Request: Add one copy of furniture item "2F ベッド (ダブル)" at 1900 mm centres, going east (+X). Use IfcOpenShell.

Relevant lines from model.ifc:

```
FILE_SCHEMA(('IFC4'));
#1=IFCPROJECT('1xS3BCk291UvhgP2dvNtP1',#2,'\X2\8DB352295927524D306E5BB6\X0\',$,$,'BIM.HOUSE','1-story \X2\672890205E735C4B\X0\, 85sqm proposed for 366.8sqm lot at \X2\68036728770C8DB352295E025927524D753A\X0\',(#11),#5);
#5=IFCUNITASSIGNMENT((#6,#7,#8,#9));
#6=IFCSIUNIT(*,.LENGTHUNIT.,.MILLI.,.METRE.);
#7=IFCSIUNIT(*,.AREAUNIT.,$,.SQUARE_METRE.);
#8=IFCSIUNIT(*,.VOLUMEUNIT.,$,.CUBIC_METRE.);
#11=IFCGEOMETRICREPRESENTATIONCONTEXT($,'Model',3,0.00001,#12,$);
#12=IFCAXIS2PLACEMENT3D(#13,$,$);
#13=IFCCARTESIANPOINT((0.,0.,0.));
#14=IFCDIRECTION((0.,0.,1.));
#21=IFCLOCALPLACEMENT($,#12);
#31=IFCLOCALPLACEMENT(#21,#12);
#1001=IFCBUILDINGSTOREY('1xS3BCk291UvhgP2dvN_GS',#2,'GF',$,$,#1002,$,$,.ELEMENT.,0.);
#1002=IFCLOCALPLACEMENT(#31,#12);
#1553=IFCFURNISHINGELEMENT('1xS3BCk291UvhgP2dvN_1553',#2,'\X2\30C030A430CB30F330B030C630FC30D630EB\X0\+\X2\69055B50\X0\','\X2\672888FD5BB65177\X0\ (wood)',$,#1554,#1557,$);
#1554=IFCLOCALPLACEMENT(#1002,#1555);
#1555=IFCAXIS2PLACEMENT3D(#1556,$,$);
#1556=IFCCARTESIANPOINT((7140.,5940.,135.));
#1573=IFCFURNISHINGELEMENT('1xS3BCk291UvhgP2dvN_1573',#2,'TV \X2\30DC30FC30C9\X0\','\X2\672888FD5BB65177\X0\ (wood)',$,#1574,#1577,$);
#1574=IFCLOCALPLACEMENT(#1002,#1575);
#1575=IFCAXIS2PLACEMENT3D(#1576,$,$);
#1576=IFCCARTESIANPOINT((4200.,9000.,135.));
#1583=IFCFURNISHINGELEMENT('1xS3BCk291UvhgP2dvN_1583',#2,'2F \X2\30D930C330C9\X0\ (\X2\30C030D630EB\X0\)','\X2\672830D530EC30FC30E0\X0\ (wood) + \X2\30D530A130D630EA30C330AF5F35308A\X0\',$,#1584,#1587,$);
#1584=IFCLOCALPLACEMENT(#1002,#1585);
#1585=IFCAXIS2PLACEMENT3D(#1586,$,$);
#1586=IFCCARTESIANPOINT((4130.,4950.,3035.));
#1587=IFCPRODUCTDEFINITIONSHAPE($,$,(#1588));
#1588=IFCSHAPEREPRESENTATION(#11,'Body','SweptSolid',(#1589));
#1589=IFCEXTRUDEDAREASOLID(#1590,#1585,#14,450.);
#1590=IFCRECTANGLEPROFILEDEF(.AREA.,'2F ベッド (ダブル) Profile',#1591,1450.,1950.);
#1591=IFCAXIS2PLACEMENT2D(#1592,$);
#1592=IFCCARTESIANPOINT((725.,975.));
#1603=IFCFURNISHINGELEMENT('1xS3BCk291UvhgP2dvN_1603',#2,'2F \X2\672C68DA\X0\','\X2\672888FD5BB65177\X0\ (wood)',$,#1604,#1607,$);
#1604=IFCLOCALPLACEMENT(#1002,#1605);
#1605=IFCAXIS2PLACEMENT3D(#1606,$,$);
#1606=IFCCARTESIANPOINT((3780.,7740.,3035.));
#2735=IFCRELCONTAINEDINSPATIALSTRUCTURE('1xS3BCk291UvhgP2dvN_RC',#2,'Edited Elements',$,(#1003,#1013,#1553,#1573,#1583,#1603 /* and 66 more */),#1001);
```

```python
import numpy as np
import ifcopenshell
import ifcopenshell.api.geometry
import ifcopenshell.api.root
import ifcopenshell.util.element
import ifcopenshell.util.placement
import ifcopenshell.util.unit

model = ifcopenshell.open("model.ifc")
unit_scale = ifcopenshell.util.unit.calculate_unit_scale(model)


def reuse_history(source, copy):
    """copy_class also copies each property set's owner history, people and application; keep the originals."""
    for rel in copy.IsDefinedBy:
        if rel.is_a("IfcRelDefinesByProperties") and (history := rel.RelatingPropertyDefinition.OwnerHistory):
            rel.RelatingPropertyDefinition.OwnerHistory = source.OwnerHistory
            ifcopenshell.util.element.remove_deep2(model, history)


source = model.by_guid("1xS3BCk291UvhgP2dvN_1583")
base = ifcopenshell.util.placement.get_local_placement(source.ObjectPlacement)
step = np.array([1.0, 0.0, 0.0]) * 1.9 / unit_scale

for i in range(1, 2):
    copy = ifcopenshell.api.root.copy_class(model, product=source)
    copy.Representation = ifcopenshell.util.element.copy_deep(
        model, source.Representation, exclude=["IfcGeometricRepresentationContext", "IfcRepresentationMap"]
    )
    reuse_history(source, copy)
    matrix = base.copy()
    matrix[:3, 3] += i * step
    print("added at", matrix[:3, 3].round(3) + 0.0)
    ifcopenshell.api.geometry.edit_object_placement(model, product=copy, matrix=matrix, is_si=False)

model.write("model_v2.ifc")
```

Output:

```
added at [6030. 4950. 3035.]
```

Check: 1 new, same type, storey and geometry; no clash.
